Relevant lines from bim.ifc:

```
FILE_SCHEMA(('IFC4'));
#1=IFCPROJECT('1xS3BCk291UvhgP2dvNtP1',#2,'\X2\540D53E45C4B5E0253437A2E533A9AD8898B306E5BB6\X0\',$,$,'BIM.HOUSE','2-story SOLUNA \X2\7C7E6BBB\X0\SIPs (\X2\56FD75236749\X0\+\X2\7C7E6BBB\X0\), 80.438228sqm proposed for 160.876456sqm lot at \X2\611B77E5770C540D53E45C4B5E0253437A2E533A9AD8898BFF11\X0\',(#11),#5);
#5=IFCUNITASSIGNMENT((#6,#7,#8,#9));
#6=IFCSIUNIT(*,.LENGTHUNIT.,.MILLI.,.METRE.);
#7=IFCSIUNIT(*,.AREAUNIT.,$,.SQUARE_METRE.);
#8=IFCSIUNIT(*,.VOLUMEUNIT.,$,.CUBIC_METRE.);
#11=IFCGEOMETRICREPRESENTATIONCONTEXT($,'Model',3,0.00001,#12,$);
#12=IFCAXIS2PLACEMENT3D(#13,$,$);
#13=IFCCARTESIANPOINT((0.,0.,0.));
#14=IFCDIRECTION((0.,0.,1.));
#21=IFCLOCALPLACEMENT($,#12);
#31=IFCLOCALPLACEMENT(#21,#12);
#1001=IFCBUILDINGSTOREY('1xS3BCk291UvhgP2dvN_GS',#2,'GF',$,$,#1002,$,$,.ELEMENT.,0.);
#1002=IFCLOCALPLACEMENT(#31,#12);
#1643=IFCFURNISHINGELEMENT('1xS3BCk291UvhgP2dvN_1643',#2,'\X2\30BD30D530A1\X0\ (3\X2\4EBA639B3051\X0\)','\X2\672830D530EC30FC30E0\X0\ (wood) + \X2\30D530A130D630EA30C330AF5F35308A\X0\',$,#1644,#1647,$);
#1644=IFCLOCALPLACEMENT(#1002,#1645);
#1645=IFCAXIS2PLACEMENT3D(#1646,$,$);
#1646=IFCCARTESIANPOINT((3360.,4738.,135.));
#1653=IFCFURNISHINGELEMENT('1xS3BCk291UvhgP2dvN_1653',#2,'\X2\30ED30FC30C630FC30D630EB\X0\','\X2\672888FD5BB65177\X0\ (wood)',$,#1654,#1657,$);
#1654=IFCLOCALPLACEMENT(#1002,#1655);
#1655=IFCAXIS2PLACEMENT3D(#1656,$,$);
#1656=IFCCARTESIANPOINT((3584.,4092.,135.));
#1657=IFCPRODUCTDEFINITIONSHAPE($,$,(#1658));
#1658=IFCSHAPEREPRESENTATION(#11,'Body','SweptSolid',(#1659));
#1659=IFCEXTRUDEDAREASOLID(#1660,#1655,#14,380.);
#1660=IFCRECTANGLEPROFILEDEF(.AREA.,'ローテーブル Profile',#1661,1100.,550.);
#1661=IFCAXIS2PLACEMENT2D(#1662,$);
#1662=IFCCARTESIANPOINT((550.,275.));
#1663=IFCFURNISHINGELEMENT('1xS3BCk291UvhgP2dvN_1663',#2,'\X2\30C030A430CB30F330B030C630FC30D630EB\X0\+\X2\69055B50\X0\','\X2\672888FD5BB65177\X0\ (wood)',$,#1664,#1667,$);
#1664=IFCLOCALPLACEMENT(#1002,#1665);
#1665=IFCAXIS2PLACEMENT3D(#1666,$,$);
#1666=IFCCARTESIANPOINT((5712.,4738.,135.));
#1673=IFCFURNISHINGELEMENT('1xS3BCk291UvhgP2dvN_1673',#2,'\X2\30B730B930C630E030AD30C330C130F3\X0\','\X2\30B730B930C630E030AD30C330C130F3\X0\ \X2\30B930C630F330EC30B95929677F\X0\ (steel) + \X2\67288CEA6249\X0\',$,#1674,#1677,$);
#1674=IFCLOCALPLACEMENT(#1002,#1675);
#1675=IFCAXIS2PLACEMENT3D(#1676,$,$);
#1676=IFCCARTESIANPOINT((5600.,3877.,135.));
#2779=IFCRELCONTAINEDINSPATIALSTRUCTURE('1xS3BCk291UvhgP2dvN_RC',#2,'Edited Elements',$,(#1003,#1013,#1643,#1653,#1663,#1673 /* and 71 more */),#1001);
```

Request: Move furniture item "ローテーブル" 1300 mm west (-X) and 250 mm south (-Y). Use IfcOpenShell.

```python
import ifcopenshell
import ifcopenshell.api.geometry
import ifcopenshell.util.placement

model = ifcopenshell.open("bim.ifc")

item = model.by_guid("1xS3BCk291UvhgP2dvN_1653")
matrix = ifcopenshell.util.placement.get_local_placement(item.ObjectPlacement)
matrix[0, 3] -= 1300.0
matrix[1, 3] -= 250.0
ifcopenshell.api.geometry.edit_object_placement(model, product=item, matrix=matrix, is_si=False)

print(ifcopenshell.util.placement.get_local_placement(item.ObjectPlacement).round(3) + 0.0)

model.write("bim-out.ifc")
```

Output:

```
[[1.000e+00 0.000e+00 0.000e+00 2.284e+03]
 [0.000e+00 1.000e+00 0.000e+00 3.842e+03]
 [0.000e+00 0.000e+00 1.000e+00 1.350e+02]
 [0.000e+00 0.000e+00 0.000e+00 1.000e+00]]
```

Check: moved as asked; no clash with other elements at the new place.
